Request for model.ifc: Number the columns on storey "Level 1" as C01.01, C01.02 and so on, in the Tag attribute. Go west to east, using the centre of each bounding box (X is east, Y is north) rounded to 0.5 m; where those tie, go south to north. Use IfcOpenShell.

First a look at what the model holds.

```python
import ifcopenshell
import ifcopenshell.util.element
import ifcopenshell.util.placement

model = ifcopenshell.open("model.ifc")
print(model.schema)
storey = next(s for s in model.by_type("IfcBuildingStorey") if s.Name == "Level 1")
columns = [e for e in ifcopenshell.util.element.get_decomposition(storey) if e.is_a("IfcColumn")]
for e in sorted(columns, key=lambda e: e.id()):
    origin = ifcopenshell.util.placement.get_local_placement(e.ObjectPlacement)[:3, 3]
    print(e.id(), e.Tag, e.Name, origin.round(2) + 0.0, sep=" | ")
```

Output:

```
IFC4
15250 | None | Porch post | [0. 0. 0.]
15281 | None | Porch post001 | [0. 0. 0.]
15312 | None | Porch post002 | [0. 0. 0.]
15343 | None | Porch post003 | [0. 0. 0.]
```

```python
import ifcopenshell
import ifcopenshell.geom
import ifcopenshell.util.element
import ifcopenshell.util.shape

model = ifcopenshell.open("model.ifc")
settings = ifcopenshell.geom.settings()
settings.set("use-world-coords", True)


def centre(element):
    shape = ifcopenshell.geom.create_shape(settings, element)
    return ifcopenshell.util.shape.get_bbox_centroid(shape.geometry)


storey = next(s for s in model.by_type("IfcBuildingStorey") if s.Name == "Level 1")
columns = [e for e in ifcopenshell.util.element.get_decomposition(storey) if e.is_a("IfcColumn")]

# Insertion points can sit at a corner or the storey origin, so sort by the geometry (in metres).
centres = {e: centre(e) for e in columns}
columns.sort(key=lambda e: (round(centres[e][0] / 0.5), centres[e][1]))

for i, e in enumerate(columns, start=1):
    number = f"C01.{i:02d}"
    e.Tag = number
    print(e.id(), number)

model.write("model_v2.ifc")
```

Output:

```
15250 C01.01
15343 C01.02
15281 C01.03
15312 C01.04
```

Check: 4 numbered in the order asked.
